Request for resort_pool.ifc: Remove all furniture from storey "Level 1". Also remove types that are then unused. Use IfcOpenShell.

First a look at what the model holds.

```python
import ifcopenshell
import ifcopenshell.util.element

model = ifcopenshell.open("resort_pool.ifc")
print(model.schema)
storey = next(s for s in model.by_type("IfcBuildingStorey") if s.Name == "Level 1")
furniture = [e for e in ifcopenshell.util.element.get_decomposition(storey) if e.is_a("IfcFurnishingElement")]
seen = {}
for e in furniture:
    element_type = ifcopenshell.util.element.get_type(e)
    name = element_type.Name if element_type not in (None, e) else None
    seen[name] = seen.get(name, 0) + 1
for name, count in sorted(seen.items(), key=str):
    print(count, "x", name)
```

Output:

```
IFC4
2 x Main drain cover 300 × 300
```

```python
import ifcopenshell
import ifcopenshell.api.root
import ifcopenshell.util.element

model = ifcopenshell.open("resort_pool.ifc")

storey = next(s for s in model.by_type("IfcBuildingStorey") if s.Name == "Level 1")
furniture = [e for e in ifcopenshell.util.element.get_decomposition(storey) if e.is_a("IfcFurnishingElement")]
types = {ifcopenshell.util.element.get_type(e) for e in furniture} - {None, *furniture}

for e in furniture:
    ifcopenshell.api.root.remove_product(model, product=e)
print(len(furniture), "removed")

unused = [t for t in types if not ifcopenshell.util.element.get_types(t)]
for t in unused:
    ifcopenshell.api.root.remove_product(model, product=t)
print(len(unused), "unused types removed")

model.write("resort_pool_edited.ifc")
```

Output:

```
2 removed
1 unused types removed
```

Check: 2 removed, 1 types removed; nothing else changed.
